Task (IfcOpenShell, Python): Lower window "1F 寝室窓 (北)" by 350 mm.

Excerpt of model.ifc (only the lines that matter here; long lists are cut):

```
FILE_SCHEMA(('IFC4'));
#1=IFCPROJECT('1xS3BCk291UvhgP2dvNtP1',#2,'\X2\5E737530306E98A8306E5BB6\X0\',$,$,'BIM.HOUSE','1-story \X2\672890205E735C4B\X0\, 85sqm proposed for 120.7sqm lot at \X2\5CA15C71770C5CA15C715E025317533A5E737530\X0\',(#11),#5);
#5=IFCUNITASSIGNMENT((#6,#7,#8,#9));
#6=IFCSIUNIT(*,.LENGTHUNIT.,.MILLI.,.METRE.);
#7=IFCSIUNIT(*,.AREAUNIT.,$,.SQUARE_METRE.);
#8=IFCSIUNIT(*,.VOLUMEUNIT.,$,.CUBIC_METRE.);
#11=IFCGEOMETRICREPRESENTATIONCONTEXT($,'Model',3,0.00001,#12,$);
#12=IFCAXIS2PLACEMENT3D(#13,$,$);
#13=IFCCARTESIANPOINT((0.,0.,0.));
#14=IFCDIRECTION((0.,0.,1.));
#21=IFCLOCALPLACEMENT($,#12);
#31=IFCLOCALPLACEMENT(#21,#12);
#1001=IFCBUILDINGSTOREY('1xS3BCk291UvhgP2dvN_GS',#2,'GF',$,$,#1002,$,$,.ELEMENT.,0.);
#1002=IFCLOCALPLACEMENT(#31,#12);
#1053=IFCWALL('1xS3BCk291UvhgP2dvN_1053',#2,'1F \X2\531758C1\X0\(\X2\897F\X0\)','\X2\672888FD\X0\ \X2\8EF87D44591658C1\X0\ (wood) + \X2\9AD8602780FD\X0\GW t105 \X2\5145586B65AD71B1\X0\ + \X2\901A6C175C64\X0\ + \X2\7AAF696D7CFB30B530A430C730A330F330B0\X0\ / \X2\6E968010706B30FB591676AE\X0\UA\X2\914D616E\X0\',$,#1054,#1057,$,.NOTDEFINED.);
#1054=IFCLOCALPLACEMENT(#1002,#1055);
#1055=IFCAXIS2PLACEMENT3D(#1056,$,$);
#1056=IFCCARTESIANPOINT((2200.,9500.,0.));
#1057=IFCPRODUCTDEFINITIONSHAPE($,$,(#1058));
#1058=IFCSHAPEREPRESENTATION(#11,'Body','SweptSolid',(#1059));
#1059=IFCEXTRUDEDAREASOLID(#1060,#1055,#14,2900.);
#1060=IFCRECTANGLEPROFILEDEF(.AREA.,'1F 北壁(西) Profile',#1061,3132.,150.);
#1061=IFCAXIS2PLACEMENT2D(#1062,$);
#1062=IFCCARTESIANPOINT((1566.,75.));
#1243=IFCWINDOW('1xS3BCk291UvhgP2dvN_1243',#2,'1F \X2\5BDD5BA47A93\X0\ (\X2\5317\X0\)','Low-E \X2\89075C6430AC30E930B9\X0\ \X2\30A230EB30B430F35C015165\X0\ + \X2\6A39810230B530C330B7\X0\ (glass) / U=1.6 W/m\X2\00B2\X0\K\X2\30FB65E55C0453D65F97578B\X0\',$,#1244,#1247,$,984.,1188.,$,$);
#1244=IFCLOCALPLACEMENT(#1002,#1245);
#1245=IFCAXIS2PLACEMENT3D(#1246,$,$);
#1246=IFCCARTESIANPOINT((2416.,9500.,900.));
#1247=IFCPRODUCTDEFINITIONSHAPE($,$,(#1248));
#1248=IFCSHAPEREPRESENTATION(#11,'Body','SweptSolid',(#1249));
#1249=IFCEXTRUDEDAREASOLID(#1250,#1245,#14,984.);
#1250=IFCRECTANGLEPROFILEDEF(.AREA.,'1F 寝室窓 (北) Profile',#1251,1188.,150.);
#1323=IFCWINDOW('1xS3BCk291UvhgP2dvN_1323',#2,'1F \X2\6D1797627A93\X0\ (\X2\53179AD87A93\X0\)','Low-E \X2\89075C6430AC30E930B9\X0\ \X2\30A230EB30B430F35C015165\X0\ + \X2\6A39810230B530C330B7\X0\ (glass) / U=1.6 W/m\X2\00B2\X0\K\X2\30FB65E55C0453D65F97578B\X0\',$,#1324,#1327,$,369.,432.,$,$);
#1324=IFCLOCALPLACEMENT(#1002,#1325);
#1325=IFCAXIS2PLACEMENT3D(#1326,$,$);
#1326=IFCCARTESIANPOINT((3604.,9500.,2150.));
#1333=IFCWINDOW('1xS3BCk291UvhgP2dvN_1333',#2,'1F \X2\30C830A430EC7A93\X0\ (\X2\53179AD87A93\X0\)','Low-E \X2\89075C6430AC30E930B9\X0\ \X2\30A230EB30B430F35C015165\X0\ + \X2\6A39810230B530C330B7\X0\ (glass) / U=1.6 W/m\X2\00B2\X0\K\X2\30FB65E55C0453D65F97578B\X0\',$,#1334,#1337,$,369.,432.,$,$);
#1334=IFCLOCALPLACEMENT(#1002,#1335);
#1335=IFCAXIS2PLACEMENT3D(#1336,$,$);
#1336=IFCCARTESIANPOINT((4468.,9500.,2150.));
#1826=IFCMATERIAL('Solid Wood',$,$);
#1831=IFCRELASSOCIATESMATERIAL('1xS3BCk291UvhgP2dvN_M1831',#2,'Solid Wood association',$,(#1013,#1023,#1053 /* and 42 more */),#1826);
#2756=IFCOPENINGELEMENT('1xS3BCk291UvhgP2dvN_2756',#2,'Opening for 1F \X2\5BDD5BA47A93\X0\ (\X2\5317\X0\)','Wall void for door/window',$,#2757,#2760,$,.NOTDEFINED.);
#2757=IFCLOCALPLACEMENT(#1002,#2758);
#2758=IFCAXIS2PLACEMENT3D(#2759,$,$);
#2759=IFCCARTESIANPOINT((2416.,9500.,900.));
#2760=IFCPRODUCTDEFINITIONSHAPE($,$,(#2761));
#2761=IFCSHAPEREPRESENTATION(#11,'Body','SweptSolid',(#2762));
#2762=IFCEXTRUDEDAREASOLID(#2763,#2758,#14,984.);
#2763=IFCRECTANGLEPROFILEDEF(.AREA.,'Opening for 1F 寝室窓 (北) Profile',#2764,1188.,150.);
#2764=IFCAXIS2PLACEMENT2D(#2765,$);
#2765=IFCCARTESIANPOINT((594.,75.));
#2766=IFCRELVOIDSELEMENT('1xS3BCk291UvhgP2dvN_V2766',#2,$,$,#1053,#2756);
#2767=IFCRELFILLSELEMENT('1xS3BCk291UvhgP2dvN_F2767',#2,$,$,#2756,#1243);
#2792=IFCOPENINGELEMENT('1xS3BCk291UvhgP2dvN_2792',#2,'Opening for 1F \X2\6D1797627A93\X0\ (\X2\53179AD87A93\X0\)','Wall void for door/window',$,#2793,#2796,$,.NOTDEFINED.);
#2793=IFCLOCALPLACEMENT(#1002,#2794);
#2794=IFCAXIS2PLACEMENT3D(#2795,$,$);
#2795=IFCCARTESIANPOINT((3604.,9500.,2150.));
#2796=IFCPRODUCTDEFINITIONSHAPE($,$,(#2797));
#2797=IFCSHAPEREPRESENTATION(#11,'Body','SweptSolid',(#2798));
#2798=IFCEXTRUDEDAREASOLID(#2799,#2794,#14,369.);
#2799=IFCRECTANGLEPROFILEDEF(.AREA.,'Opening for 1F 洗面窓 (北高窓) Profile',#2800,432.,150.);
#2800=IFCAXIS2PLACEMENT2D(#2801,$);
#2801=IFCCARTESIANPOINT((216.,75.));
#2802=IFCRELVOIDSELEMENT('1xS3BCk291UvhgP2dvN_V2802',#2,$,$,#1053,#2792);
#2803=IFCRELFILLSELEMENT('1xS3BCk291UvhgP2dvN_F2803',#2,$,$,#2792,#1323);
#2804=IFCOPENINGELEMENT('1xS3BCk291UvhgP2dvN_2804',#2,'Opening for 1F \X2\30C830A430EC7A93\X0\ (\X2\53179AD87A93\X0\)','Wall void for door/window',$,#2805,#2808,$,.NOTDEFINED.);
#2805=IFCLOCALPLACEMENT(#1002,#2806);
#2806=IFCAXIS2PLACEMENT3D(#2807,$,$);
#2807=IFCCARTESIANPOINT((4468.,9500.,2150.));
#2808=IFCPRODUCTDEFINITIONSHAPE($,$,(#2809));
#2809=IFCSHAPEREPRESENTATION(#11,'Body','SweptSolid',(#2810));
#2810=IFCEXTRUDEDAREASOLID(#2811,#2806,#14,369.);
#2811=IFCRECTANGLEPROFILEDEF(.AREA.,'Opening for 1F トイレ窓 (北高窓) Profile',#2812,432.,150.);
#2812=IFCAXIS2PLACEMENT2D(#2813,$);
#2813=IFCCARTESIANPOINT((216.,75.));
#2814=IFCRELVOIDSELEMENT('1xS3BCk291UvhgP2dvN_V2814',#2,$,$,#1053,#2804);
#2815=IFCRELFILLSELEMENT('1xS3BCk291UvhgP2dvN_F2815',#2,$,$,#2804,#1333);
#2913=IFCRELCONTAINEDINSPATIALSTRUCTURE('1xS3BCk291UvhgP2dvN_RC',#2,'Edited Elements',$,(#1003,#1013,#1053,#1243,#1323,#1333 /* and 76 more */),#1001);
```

```python
import numpy as np
import ifcopenshell
import ifcopenshell.api.geometry
import ifcopenshell.util.placement
import ifcopenshell.util.unit

model = ifcopenshell.open("model.ifc")
unit_scale = ifcopenshell.util.unit.calculate_unit_scale(model)

window = model.by_guid("1xS3BCk291UvhgP2dvN_1243")
opening = window.FillsVoids[0].RelatingOpeningElement
dz = -0.35 / unit_scale

shift = np.array([0.0, 0.0, dz])
# The window is not placed relative to its opening, so move both.
for product in (opening, window):
    matrix = ifcopenshell.util.placement.get_local_placement(product.ObjectPlacement)
    matrix[:3, 3] += shift
    ifcopenshell.api.geometry.edit_object_placement(model, product=product, matrix=matrix, is_si=False)

print(f"moved by {dz * unit_scale:+.3f} m")

model.write("model_v2.ifc")
```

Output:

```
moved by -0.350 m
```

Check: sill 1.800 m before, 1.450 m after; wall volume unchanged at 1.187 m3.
